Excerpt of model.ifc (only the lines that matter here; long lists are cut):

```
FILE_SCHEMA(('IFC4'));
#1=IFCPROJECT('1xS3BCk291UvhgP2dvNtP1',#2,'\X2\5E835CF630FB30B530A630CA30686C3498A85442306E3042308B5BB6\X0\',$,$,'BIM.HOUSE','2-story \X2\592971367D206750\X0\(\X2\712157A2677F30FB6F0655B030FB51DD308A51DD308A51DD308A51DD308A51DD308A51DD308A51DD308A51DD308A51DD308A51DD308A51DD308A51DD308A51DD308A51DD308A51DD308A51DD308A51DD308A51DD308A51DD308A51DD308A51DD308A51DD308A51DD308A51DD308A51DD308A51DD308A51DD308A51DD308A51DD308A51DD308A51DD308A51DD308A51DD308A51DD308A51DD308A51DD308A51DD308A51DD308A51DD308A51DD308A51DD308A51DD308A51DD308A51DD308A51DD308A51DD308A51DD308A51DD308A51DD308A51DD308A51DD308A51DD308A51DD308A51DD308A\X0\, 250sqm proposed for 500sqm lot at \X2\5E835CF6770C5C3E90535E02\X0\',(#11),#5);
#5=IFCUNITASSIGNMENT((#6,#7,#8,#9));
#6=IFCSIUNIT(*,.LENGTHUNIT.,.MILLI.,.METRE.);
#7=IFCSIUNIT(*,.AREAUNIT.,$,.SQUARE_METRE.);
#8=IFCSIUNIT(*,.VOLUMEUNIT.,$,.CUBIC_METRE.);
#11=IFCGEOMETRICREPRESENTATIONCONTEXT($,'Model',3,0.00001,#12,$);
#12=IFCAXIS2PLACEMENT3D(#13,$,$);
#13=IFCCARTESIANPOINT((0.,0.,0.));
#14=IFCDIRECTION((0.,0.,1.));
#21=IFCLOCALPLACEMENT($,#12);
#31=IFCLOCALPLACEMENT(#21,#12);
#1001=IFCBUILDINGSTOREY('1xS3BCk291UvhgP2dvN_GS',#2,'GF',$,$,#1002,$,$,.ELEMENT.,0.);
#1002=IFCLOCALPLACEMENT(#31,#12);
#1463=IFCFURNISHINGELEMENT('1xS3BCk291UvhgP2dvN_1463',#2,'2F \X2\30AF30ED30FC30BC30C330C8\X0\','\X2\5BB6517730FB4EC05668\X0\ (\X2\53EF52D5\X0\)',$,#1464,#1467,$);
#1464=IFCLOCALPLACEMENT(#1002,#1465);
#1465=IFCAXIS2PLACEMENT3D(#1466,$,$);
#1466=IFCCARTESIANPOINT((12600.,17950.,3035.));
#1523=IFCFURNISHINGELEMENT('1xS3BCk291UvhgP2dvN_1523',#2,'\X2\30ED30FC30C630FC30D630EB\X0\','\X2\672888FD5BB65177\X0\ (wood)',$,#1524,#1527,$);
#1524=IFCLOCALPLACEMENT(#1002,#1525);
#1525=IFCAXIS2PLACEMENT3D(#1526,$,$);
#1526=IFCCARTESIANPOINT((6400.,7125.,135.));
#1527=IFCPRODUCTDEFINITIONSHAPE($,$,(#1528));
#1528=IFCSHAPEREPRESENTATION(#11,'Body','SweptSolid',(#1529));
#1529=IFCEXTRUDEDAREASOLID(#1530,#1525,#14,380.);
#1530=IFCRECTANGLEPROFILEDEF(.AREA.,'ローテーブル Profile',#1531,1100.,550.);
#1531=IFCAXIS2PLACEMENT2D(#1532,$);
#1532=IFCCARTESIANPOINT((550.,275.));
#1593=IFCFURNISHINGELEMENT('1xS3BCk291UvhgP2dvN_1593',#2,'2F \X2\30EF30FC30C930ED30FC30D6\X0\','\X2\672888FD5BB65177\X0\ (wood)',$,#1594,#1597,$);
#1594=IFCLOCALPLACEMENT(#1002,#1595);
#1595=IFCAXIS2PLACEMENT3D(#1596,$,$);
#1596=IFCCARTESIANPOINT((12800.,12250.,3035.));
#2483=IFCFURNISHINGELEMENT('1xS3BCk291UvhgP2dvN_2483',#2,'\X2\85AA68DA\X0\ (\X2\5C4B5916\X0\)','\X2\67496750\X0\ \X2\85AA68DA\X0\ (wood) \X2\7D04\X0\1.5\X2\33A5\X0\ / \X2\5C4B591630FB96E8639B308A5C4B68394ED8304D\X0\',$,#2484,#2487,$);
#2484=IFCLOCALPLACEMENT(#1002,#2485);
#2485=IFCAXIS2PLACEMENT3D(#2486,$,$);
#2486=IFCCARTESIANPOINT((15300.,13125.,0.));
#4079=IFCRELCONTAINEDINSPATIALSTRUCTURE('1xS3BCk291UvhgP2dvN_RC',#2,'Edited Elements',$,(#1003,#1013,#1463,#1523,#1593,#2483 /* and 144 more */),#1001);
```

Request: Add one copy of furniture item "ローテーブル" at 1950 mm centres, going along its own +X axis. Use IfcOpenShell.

```python
import ifcopenshell
import ifcopenshell.api.geometry
import ifcopenshell.api.root
import ifcopenshell.util.element
import ifcopenshell.util.placement
import ifcopenshell.util.unit

model = ifcopenshell.open("model.ifc")
unit_scale = ifcopenshell.util.unit.calculate_unit_scale(model)


def reuse_history(source, copy):
    """copy_class also copies each property set's owner history, people and application; keep the originals."""
    for rel in copy.IsDefinedBy:
        if rel.is_a("IfcRelDefinesByProperties") and (history := rel.RelatingPropertyDefinition.OwnerHistory):
            rel.RelatingPropertyDefinition.OwnerHistory = source.OwnerHistory
            ifcopenshell.util.element.remove_deep2(model, history)


source = model.by_id(1523)
base = ifcopenshell.util.placement.get_local_placement(source.ObjectPlacement)
step = base[:3, 0] * 1.95 / unit_scale

for i in range(1, 2):
    copy = ifcopenshell.api.root.copy_class(model, product=source)
    copy.Representation = ifcopenshell.util.element.copy_deep(
        model, source.Representation, exclude=["IfcGeometricRepresentationContext", "IfcRepresentationMap"]
    )
    reuse_history(source, copy)
    matrix = base.copy()
    matrix[:3, 3] += i * step
    print("added at", matrix[:3, 3].round(3) + 0.0)
    ifcopenshell.api.geometry.edit_object_placement(model, product=copy, matrix=matrix, is_si=False)

model.write("model_updated.ifc")
```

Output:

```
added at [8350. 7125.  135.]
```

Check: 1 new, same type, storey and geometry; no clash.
